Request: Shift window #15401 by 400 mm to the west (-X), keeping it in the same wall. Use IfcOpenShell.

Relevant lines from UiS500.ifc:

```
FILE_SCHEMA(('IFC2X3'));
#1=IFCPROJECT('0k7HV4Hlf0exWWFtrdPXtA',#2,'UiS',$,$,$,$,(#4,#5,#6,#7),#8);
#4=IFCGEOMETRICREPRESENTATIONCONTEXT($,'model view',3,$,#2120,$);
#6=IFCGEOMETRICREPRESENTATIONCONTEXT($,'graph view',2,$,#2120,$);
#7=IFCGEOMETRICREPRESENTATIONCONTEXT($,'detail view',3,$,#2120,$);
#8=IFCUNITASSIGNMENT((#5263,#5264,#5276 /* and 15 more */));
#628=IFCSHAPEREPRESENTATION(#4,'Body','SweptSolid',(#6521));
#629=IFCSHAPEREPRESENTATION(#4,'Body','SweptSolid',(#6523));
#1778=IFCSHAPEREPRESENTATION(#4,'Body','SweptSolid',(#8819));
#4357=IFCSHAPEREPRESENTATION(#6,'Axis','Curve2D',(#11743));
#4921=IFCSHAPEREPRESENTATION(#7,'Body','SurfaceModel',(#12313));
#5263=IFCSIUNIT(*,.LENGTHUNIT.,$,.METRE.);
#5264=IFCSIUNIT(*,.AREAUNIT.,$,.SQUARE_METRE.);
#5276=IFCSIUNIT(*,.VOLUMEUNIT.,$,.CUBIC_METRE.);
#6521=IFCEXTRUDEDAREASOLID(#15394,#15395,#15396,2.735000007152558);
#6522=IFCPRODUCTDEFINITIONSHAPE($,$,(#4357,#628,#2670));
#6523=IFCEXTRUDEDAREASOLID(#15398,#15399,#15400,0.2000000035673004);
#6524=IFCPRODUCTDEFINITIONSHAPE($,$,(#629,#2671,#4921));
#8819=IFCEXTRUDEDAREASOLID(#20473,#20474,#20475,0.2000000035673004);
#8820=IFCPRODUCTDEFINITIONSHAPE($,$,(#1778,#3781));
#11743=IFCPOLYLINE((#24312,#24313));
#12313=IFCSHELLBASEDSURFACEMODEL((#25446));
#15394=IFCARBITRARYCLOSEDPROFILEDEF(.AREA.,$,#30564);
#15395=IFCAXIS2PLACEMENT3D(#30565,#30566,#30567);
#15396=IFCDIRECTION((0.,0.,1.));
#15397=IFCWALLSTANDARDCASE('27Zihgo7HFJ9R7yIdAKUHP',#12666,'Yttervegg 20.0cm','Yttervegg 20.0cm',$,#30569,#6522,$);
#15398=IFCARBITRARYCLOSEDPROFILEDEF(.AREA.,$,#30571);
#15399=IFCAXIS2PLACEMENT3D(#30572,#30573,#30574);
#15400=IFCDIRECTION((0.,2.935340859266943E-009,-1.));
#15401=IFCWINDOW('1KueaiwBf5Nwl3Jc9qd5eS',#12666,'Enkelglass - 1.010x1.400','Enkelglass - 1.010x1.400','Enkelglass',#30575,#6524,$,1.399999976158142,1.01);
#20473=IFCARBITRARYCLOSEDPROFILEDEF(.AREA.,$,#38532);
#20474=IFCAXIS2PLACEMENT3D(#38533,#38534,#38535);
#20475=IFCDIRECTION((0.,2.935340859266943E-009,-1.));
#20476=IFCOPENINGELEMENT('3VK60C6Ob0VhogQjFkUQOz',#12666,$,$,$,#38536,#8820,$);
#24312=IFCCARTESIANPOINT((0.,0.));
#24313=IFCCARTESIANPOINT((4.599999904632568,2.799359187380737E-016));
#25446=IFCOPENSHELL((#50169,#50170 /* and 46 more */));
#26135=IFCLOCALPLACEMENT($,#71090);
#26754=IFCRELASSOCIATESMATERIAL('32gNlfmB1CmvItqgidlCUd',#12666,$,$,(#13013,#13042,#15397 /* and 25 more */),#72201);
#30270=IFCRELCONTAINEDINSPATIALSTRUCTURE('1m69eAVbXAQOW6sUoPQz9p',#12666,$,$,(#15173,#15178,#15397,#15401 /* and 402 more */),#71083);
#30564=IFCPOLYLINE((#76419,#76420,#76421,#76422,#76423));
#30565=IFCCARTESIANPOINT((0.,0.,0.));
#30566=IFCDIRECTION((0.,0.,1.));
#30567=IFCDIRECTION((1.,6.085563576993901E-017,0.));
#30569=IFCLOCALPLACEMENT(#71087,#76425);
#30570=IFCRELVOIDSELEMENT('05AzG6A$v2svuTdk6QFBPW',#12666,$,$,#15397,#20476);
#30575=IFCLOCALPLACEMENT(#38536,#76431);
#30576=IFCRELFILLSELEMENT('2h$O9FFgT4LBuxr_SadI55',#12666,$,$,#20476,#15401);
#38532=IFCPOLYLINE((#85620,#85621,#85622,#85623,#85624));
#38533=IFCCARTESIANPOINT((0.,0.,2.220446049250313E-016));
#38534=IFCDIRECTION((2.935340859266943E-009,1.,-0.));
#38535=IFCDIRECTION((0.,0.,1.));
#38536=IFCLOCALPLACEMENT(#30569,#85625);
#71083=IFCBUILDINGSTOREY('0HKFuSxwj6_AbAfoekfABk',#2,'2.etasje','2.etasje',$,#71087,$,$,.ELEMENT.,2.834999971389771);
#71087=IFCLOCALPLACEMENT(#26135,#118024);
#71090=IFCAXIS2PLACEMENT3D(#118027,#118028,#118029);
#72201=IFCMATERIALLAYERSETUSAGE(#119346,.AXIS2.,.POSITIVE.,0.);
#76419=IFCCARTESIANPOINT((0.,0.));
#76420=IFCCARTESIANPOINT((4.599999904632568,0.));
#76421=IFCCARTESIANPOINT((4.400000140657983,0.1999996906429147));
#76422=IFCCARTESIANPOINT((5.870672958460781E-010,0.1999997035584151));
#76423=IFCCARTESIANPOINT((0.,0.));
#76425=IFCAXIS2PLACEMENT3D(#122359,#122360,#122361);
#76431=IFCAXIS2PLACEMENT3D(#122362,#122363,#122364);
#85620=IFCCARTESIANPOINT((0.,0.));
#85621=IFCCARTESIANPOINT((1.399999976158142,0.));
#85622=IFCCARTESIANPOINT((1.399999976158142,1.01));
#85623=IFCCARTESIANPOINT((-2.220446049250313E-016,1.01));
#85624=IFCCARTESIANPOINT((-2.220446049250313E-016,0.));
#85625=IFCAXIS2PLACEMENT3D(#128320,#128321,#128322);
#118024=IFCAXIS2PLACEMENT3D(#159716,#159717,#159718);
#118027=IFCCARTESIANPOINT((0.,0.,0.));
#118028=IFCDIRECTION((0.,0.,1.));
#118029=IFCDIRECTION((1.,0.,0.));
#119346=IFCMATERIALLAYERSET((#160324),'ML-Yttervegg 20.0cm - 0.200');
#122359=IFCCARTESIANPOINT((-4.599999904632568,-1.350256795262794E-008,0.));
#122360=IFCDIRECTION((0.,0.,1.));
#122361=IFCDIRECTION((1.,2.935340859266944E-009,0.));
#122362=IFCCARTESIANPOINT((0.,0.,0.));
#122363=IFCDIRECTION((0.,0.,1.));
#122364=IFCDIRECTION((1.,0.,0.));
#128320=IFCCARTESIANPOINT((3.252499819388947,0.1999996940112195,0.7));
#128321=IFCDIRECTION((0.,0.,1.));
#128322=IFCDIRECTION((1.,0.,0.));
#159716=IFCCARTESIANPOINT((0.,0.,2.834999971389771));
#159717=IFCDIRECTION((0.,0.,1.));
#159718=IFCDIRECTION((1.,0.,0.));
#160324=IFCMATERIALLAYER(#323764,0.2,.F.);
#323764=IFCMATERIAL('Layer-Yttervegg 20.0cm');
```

```python
import ifcopenshell
import ifcopenshell.api.geometry
import ifcopenshell.util.placement

model = ifcopenshell.open("UiS500.ifc")

window = model.by_guid("1KueaiwBf5Nwl3Jc9qd5eS")
opening = window.FillsVoids[0].RelatingOpeningElement
wall = opening.VoidsElements[0].RelatingBuildingElement

wall_matrix = ifcopenshell.util.placement.get_local_placement(wall.ObjectPlacement)
shift = wall_matrix[:3, 0] * -0.4
before = ifcopenshell.util.placement.get_local_placement(window.ObjectPlacement)[:3, 3].copy()

# The window is placed relative to its opening, so it follows when the opening moves.
matrix = ifcopenshell.util.placement.get_local_placement(opening.ObjectPlacement)
matrix[:3, 3] += shift
ifcopenshell.api.geometry.edit_object_placement(
    model, product=opening, matrix=matrix, is_si=False, should_transform_children=True
)

after = ifcopenshell.util.placement.get_local_placement(window.ObjectPlacement)[:3, 3]
print("window moved by", (after - before).round(3) + 0.0)

model.write("UiS500_v2.ifc")
```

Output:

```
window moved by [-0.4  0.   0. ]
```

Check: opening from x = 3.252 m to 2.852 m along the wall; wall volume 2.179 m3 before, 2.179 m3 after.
